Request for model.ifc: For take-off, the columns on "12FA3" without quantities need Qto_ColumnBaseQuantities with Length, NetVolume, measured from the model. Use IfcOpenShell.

First a look at what the model holds.

```python
import ifcopenshell
import ifcopenshell.util.element
import ifcopenshell.util.unit

model = ifcopenshell.open("model.ifc")
print(model.schema)
for unit_type in ("LENGTHUNIT", "AREAUNIT", "VOLUMEUNIT"):
    print(unit_type, ifcopenshell.util.unit.calculate_unit_scale(model, unit_type))
storey = next(s for s in model.by_type("IfcBuildingStorey") if s.Name == "12FA3")
columns = [e for e in ifcopenshell.util.element.get_decomposition(storey) if e.is_a("IfcColumn")]
for e in sorted(columns, key=lambda e: e.id()):
    print(e.id(), e.is_a(), e.Name, list(ifcopenshell.util.element.get_psets(e, qtos_only=True)), sep=" | ")
```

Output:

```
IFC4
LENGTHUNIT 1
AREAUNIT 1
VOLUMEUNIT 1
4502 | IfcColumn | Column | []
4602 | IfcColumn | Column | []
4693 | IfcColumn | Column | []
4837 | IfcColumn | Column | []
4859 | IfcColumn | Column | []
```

```python
import ifcopenshell
import ifcopenshell.api.pset
import ifcopenshell.geom
import ifcopenshell.util.element
import ifcopenshell.util.shape
import ifcopenshell.util.unit

model = ifcopenshell.open("model.ifc")
unit_scale = ifcopenshell.util.unit.calculate_unit_scale(model)
volume_scale = ifcopenshell.util.unit.calculate_unit_scale(model, "VOLUMEUNIT")
settings = ifcopenshell.geom.settings()

storey = next(s for s in model.by_type("IfcBuildingStorey") if s.Name == "12FA3")
columns = [e for e in ifcopenshell.util.element.get_decomposition(storey) if e.is_a("IfcColumn")]

for e in sorted(columns, key=lambda e: e.id()):
    if ifcopenshell.util.element.get_psets(e, qtos_only=True, should_inherit=False):
        continue
    # Geometry comes back in metres, in the element's own axes.
    shape = ifcopenshell.geom.create_shape(settings, e)
    values = {
        "Length": ifcopenshell.util.shape.get_z(shape.geometry) / unit_scale,
        "NetVolume": ifcopenshell.util.shape.get_volume(shape.geometry) / volume_scale,
    }
    qto = ifcopenshell.api.pset.add_qto(model, product=e, name="Qto_ColumnBaseQuantities")
    ifcopenshell.api.pset.edit_qto(model, qto=qto, properties=values)
    print(e.id(), {k: round(v, 3) for k, v in values.items()})

model.write("model_v2.ifc")
```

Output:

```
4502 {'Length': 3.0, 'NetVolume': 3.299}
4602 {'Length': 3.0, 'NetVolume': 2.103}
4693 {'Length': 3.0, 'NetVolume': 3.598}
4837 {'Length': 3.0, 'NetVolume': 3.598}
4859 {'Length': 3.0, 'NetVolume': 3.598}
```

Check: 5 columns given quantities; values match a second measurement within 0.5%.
